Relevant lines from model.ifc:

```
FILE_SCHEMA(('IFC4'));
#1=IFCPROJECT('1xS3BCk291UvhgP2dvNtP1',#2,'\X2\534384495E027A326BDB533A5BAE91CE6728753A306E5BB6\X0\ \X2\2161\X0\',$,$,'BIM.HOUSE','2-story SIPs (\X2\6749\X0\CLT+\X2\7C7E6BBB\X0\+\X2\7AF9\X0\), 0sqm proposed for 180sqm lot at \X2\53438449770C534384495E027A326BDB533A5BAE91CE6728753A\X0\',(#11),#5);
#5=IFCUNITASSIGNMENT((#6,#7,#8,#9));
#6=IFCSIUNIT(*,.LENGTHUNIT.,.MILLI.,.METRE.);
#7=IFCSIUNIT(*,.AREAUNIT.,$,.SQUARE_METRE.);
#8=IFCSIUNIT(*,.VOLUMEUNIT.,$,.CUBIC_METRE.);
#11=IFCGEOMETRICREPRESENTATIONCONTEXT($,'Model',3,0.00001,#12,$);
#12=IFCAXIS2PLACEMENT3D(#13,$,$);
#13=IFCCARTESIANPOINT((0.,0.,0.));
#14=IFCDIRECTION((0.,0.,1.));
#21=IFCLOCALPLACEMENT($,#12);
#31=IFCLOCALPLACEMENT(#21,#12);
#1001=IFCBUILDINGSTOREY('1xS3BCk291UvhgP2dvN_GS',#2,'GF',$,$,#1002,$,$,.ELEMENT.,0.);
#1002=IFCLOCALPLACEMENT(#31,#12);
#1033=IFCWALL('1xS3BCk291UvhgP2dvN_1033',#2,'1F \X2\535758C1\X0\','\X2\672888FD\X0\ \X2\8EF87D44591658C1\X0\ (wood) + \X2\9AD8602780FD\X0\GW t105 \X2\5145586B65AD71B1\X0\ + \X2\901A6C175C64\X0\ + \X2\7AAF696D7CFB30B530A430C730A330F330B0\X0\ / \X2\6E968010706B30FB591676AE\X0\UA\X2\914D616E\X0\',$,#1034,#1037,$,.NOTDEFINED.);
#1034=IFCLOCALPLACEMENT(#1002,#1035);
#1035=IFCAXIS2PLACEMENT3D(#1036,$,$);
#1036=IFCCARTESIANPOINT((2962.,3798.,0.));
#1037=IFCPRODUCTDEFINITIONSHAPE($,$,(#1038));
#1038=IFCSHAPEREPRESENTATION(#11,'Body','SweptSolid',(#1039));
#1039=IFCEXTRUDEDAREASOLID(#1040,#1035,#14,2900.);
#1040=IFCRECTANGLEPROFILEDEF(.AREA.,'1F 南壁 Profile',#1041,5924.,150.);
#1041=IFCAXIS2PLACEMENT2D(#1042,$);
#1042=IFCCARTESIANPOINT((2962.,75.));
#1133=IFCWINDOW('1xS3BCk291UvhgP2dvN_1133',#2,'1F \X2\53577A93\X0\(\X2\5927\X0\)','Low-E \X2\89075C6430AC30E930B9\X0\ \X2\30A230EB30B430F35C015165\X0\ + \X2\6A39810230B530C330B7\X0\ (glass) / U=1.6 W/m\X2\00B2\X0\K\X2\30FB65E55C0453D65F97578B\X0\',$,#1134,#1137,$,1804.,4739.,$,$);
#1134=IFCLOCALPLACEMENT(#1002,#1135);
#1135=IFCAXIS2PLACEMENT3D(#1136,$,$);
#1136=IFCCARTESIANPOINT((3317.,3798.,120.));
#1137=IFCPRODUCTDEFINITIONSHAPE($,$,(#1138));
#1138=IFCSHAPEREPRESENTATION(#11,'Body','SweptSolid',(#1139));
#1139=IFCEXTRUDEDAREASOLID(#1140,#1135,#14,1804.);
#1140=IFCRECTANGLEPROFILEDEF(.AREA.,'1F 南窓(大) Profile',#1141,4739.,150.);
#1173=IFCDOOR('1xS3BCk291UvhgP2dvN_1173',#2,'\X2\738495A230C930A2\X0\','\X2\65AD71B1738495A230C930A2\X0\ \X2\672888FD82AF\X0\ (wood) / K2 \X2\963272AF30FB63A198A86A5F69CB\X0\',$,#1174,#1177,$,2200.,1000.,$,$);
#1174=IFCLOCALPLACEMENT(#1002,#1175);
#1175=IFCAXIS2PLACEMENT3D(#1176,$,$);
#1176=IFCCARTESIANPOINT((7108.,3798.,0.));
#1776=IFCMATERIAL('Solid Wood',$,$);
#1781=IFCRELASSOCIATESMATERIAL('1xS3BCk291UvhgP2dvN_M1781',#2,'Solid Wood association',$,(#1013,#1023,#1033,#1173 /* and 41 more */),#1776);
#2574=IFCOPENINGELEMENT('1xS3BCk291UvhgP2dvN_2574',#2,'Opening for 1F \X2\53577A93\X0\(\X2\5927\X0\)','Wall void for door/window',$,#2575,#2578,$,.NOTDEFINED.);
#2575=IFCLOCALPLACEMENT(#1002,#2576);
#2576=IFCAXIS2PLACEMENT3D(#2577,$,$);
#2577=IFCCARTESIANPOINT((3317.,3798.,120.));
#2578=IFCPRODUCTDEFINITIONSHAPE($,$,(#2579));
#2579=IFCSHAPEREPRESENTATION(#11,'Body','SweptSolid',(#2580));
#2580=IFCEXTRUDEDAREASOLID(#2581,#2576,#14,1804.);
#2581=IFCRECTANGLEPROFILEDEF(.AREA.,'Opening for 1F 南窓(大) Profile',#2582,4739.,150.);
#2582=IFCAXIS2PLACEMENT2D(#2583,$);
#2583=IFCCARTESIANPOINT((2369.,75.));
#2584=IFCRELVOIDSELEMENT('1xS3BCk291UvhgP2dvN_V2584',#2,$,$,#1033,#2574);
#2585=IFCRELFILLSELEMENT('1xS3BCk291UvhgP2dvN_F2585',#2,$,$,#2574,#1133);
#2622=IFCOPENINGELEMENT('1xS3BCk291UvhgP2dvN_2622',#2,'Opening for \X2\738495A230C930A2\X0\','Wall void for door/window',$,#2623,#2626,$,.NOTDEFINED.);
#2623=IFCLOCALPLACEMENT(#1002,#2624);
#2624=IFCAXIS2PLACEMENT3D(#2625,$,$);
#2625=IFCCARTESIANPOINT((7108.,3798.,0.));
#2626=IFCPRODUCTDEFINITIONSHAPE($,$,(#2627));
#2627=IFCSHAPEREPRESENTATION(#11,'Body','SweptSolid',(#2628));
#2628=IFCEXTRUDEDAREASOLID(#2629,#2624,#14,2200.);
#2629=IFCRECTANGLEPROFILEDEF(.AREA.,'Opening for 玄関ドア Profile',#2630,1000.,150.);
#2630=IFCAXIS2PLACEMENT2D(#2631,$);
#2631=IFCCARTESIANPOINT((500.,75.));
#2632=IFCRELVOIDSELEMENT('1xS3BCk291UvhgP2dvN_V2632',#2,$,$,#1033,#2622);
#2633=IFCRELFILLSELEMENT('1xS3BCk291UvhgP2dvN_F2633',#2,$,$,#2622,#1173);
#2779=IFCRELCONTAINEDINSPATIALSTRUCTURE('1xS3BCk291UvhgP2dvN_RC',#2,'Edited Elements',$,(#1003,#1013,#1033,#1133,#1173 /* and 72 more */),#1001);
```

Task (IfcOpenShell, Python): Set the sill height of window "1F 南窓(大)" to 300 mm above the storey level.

```python
import numpy as np
import ifcopenshell
import ifcopenshell.api.geometry
import ifcopenshell.geom
import ifcopenshell.util.element
import ifcopenshell.util.placement
import ifcopenshell.util.shape
import ifcopenshell.util.unit

model = ifcopenshell.open("model.ifc")
unit_scale = ifcopenshell.util.unit.calculate_unit_scale(model)

window = model.by_guid("1xS3BCk291UvhgP2dvN_1133")
opening = window.FillsVoids[0].RelatingOpeningElement
storey = ifcopenshell.util.element.get_container(window, ifc_class="IfcBuildingStorey")
level = ifcopenshell.util.placement.get_local_placement(storey.ObjectPlacement)[2, 3]

# The opening's origin need not be at the sill, so measure its lowest point.
shape = ifcopenshell.geom.create_shape(ifcopenshell.geom.settings(), opening)
bottom = ifcopenshell.util.shape.get_shape_bottom_elevation(shape, shape.geometry) / unit_scale
dz = level + 0.3 / unit_scale - bottom

shift = np.array([0.0, 0.0, dz])
# The window is not placed relative to its opening, so move both.
for product in (opening, window):
    matrix = ifcopenshell.util.placement.get_local_placement(product.ObjectPlacement)
    matrix[:3, 3] += shift
    ifcopenshell.api.geometry.edit_object_placement(model, product=product, matrix=matrix, is_si=False)

print(f"moved by {dz * unit_scale:+.3f} m")

model.write("model-out.ifc")
```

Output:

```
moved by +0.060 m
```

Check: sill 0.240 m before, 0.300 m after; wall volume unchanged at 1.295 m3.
